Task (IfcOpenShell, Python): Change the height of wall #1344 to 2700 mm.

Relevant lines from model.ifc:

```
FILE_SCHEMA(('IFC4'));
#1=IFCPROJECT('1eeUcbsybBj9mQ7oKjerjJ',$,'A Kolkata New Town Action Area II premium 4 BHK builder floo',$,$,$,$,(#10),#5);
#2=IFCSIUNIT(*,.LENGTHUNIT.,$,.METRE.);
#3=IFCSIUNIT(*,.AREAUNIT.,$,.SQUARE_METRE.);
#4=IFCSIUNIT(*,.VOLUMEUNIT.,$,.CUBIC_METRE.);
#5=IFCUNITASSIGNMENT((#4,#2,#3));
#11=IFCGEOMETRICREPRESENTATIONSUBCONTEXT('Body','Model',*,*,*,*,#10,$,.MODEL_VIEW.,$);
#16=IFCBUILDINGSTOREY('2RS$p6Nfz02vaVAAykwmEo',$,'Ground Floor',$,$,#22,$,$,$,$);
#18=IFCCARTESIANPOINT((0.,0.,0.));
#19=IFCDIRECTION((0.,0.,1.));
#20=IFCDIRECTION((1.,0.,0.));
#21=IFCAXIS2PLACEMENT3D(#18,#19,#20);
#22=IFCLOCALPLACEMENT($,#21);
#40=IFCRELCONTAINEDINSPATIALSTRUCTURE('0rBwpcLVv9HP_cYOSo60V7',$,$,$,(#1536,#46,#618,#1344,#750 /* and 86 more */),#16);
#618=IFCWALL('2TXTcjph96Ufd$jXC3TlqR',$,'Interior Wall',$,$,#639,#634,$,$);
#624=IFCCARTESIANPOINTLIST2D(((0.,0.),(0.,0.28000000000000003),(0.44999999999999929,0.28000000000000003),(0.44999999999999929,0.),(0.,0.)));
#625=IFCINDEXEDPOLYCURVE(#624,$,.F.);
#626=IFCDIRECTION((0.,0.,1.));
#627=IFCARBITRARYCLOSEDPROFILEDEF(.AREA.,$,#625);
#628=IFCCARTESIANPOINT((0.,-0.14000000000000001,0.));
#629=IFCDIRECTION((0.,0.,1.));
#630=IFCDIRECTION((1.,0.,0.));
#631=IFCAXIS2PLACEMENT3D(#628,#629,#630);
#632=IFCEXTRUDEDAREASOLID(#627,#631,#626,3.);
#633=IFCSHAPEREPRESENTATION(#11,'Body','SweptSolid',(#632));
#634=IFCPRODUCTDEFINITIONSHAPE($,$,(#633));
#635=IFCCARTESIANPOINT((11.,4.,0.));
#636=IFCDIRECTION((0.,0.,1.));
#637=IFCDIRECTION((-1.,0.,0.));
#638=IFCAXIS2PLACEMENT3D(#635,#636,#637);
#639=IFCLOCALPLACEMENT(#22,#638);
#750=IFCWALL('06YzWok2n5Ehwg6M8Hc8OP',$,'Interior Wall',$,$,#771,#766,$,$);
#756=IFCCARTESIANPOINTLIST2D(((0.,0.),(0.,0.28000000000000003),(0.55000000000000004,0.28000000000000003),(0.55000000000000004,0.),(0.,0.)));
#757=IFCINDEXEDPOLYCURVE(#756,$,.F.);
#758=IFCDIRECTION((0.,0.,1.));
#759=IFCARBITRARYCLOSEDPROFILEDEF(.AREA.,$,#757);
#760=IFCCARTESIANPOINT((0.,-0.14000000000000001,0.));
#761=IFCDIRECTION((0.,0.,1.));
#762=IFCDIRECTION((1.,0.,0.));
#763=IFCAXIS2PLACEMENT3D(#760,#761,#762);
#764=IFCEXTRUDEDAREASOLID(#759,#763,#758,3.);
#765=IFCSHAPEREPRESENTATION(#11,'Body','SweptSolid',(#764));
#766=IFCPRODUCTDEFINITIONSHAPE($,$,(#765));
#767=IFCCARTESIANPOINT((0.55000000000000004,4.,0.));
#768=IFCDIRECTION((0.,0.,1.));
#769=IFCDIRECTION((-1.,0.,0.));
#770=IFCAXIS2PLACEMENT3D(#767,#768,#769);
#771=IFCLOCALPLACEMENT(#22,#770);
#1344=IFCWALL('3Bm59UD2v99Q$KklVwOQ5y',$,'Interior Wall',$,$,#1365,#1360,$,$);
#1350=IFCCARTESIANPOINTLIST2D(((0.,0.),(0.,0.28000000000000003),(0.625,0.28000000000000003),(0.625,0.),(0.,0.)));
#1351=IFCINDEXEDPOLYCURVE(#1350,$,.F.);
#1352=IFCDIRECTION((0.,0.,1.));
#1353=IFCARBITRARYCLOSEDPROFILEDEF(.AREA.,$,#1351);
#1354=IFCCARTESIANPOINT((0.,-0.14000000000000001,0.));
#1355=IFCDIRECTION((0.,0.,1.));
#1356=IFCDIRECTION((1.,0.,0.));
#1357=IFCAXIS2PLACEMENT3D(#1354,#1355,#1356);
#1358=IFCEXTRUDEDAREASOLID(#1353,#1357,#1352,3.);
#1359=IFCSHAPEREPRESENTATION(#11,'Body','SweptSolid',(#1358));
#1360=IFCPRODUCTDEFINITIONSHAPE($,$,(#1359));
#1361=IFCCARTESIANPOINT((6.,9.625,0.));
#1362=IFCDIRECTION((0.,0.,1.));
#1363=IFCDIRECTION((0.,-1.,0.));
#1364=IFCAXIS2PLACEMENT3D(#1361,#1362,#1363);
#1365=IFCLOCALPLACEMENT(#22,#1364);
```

```python
import ifcopenshell
import ifcopenshell.geom
import ifcopenshell.util.representation
import ifcopenshell.util.shape

model = ifcopenshell.open("model.ifc")
settings = ifcopenshell.geom.settings()


def volume(element):
    """Net volume in cubic metres, openings subtracted."""
    shape = ifcopenshell.geom.create_shape(settings, element)
    return ifcopenshell.util.shape.get_volume(shape.geometry)


wall = model.by_guid("3Bm59UD2v99Q$KklVwOQ5y")
before = volume(wall)

body = ifcopenshell.util.representation.get_representation(wall, "Model", "Body")
solid = body.Items[0]
old_height = solid.Depth
solid.Depth = 2.7
after = volume(wall)

print(f"height {old_height:g} -> {solid.Depth:g}, volume {before:.3f} -> {after:.3f} m3")

model.write("model_rev.ifc")
```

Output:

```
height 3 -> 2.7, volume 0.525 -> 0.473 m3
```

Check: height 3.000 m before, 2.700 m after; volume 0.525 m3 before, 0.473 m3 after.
